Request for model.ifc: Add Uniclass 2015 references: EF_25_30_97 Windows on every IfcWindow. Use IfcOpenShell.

First a look at what the model holds.

```python
import ifcopenshell

model = ifcopenshell.open("model.ifc")
print(model.schema)
print("classifications:", [c.Name for c in model.by_type("IfcClassification")])
for ifc_class in ("IfcDoor", "IfcRoof", "IfcStair", "IfcWall", "IfcWindow"):
    print(ifc_class, len(model.by_type(ifc_class)))
```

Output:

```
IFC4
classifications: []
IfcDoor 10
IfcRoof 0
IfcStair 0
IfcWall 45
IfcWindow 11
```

```python
import ifcopenshell
import ifcopenshell.api.classification

model = ifcopenshell.open("model.ifc")

system = ifcopenshell.api.classification.add_classification(model, classification="Uniclass 2015")

codes = {
    "IfcWindow": ("EF_25_30_97", "Windows"),
}
for ifc_class, (code, name) in codes.items():
    products = model.by_type(ifc_class)
    ifcopenshell.api.classification.add_reference(
        model, products=products, classification=system, identification=code, name=name
    )
    print(code, len(products))

model.write("model-out.ifc")
```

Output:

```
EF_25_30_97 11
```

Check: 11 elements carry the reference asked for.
